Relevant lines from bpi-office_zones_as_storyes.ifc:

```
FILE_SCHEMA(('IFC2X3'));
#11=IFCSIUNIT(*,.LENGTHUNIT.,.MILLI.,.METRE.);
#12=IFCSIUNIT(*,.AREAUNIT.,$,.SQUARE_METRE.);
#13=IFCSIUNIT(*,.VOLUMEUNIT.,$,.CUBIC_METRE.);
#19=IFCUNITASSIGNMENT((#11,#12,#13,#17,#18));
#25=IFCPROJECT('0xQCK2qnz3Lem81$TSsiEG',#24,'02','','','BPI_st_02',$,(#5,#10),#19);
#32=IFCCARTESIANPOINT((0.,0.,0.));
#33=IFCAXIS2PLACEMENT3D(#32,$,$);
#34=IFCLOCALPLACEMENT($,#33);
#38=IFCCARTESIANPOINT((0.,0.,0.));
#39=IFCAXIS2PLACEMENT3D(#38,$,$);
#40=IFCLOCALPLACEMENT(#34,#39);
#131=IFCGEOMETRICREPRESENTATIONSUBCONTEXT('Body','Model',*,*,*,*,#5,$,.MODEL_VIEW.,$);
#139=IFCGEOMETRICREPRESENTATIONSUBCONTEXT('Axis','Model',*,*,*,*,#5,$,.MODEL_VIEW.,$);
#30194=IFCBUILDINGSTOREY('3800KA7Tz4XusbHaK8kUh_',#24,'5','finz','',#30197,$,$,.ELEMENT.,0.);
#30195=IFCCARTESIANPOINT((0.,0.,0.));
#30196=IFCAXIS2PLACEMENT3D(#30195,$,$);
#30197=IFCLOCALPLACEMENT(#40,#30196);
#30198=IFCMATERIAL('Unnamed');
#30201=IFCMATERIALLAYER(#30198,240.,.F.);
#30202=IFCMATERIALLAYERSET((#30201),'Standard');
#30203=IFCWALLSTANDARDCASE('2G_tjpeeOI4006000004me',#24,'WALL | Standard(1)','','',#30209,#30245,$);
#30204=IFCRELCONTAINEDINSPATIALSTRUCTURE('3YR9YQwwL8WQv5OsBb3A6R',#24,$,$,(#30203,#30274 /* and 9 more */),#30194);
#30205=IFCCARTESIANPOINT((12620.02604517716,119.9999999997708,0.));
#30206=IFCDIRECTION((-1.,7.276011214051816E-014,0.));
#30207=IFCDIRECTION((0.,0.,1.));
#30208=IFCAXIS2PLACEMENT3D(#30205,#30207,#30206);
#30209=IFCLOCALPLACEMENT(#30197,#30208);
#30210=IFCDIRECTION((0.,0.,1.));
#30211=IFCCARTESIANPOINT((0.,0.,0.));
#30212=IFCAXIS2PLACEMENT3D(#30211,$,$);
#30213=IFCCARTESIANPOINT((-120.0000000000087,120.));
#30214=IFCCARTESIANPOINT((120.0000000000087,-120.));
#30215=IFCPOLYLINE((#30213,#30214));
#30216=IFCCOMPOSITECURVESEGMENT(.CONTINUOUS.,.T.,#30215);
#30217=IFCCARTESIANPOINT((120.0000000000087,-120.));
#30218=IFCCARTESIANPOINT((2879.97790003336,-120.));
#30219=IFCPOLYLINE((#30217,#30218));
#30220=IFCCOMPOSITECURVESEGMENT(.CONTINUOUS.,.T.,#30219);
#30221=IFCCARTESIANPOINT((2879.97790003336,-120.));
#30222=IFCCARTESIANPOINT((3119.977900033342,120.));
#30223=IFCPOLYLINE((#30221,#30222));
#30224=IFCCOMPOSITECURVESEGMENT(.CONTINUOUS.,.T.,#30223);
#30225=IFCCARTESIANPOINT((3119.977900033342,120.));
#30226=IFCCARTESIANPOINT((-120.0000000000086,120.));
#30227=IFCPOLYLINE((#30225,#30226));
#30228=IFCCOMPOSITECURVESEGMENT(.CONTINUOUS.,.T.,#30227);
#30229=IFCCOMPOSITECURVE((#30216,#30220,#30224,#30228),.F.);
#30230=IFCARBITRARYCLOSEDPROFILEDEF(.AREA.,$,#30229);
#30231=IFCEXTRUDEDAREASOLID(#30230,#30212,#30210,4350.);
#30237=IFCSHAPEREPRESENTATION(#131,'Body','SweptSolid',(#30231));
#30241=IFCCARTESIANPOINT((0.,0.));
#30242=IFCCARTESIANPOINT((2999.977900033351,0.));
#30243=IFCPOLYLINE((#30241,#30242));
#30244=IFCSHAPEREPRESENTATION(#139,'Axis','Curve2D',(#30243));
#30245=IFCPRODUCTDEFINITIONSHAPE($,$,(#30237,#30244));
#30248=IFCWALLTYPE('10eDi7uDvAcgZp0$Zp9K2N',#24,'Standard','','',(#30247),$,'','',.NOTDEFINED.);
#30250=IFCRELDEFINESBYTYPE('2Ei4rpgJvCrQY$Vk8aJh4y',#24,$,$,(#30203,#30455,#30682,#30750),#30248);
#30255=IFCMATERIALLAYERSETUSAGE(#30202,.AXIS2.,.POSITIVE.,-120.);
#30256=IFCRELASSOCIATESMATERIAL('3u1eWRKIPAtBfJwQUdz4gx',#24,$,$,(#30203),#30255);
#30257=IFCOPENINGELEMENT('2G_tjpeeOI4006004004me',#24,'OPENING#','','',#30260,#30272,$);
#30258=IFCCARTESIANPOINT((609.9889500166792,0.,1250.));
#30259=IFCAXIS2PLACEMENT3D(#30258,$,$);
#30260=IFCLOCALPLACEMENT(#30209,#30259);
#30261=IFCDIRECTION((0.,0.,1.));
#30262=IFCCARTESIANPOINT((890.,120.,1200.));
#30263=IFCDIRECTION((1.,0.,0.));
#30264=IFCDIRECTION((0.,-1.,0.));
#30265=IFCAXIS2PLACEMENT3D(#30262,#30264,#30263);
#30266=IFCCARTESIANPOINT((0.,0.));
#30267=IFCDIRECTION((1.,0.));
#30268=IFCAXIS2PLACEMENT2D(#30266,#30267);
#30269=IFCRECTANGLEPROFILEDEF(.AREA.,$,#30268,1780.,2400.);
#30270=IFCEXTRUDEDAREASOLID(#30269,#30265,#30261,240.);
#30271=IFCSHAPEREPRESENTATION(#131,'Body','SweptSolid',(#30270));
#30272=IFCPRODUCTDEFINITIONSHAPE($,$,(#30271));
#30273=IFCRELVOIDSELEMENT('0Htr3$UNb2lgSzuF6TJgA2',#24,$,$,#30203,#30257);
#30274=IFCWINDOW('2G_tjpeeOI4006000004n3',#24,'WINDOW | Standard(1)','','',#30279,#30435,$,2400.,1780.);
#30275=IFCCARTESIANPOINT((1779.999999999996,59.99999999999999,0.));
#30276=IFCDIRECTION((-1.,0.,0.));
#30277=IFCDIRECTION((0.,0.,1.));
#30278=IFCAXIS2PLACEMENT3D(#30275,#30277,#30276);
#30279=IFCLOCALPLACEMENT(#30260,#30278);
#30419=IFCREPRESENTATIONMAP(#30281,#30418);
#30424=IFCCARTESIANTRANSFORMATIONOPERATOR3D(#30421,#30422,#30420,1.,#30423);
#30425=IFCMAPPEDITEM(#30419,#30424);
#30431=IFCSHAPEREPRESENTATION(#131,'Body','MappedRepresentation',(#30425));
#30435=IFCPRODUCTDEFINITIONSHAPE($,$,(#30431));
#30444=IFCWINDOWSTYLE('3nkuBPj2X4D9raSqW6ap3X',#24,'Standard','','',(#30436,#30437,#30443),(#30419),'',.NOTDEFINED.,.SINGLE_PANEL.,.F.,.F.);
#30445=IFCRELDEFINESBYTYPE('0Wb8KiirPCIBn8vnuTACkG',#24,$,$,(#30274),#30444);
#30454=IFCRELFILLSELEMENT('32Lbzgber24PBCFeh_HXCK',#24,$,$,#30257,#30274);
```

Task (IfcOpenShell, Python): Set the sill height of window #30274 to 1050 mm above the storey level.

```python
import numpy as np
import ifcopenshell
import ifcopenshell.api.geometry
import ifcopenshell.geom
import ifcopenshell.util.element
import ifcopenshell.util.placement
import ifcopenshell.util.shape
import ifcopenshell.util.unit

model = ifcopenshell.open("bpi-office_zones_as_storyes.ifc")
unit_scale = ifcopenshell.util.unit.calculate_unit_scale(model)

window = model.by_guid("2G_tjpeeOI4006000004n3")
opening = window.FillsVoids[0].RelatingOpeningElement
storey = ifcopenshell.util.element.get_container(window, ifc_class="IfcBuildingStorey")
level = ifcopenshell.util.placement.get_local_placement(storey.ObjectPlacement)[2, 3]

# The opening's origin need not be at the sill, so measure its lowest point.
shape = ifcopenshell.geom.create_shape(ifcopenshell.geom.settings(), opening)
bottom = ifcopenshell.util.shape.get_shape_bottom_elevation(shape, shape.geometry) / unit_scale
dz = level + 1050.0 - bottom

shift = np.array([0.0, 0.0, dz])
# The window is placed relative to its opening, so it follows when the opening moves.
matrix = ifcopenshell.util.placement.get_local_placement(opening.ObjectPlacement)
matrix[:3, 3] += shift
ifcopenshell.api.geometry.edit_object_placement(
    model, product=opening, matrix=matrix, is_si=False, should_transform_children=True
)

print(f"moved by {dz * unit_scale:+.3f} m")

model.write("bpi-office_zones_as_storyes_rev.ifc")
```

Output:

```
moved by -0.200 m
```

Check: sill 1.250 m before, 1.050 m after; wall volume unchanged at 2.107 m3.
